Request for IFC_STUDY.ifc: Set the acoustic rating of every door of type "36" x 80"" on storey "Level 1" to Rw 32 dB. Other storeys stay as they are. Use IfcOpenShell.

First a look at what the model holds.

```python
import ifcopenshell
import ifcopenshell.util.element

model = ifcopenshell.open("IFC_STUDY.ifc")
print(model.schema)
storey = next(s for s in model.by_type("IfcBuildingStorey") if s.Name == "Level 1")
doors = [e for e in ifcopenshell.util.element.get_decomposition(storey) if e.is_a("IfcDoor")]
seen = {}
for e in doors:
    element_type = ifcopenshell.util.element.get_type(e)
    key = (element_type.Name if element_type != e and element_type else None, ifcopenshell.util.element.get_pset(e, "Pset_DoorCommon", "AcousticRating"))
    seen[key] = seen.get(key, 0) + 1
for (name, value), count in sorted(seen.items(), key=str):
    print(count, "x", name, "|", value)
```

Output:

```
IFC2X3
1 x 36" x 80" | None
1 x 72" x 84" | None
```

```python
import ifcopenshell
import ifcopenshell.api.pset
import ifcopenshell.util.element

model = ifcopenshell.open("IFC_STUDY.ifc")

storey = next(s for s in model.by_type("IfcBuildingStorey") if s.Name == "Level 1")
doors = [e for e in ifcopenshell.util.element.get_decomposition(storey) if e.is_a("IfcDoor")]

count = 0
for e in doors:
    element_type = ifcopenshell.util.element.get_type(e)
    if element_type in (None, e) or element_type.Name != '36" x 80"':
        continue
    # add_pset returns the element's existing set when there is one.
    pset = ifcopenshell.api.pset.add_pset(model, product=e, name="Pset_DoorCommon")
    ifcopenshell.api.pset.edit_pset(model, pset=pset, properties={"AcousticRating": "Rw 32 dB"})
    count += 1

print(count, "doors updated")

model.write("IFC_STUDY_v2.ifc")
```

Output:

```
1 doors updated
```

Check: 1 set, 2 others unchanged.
